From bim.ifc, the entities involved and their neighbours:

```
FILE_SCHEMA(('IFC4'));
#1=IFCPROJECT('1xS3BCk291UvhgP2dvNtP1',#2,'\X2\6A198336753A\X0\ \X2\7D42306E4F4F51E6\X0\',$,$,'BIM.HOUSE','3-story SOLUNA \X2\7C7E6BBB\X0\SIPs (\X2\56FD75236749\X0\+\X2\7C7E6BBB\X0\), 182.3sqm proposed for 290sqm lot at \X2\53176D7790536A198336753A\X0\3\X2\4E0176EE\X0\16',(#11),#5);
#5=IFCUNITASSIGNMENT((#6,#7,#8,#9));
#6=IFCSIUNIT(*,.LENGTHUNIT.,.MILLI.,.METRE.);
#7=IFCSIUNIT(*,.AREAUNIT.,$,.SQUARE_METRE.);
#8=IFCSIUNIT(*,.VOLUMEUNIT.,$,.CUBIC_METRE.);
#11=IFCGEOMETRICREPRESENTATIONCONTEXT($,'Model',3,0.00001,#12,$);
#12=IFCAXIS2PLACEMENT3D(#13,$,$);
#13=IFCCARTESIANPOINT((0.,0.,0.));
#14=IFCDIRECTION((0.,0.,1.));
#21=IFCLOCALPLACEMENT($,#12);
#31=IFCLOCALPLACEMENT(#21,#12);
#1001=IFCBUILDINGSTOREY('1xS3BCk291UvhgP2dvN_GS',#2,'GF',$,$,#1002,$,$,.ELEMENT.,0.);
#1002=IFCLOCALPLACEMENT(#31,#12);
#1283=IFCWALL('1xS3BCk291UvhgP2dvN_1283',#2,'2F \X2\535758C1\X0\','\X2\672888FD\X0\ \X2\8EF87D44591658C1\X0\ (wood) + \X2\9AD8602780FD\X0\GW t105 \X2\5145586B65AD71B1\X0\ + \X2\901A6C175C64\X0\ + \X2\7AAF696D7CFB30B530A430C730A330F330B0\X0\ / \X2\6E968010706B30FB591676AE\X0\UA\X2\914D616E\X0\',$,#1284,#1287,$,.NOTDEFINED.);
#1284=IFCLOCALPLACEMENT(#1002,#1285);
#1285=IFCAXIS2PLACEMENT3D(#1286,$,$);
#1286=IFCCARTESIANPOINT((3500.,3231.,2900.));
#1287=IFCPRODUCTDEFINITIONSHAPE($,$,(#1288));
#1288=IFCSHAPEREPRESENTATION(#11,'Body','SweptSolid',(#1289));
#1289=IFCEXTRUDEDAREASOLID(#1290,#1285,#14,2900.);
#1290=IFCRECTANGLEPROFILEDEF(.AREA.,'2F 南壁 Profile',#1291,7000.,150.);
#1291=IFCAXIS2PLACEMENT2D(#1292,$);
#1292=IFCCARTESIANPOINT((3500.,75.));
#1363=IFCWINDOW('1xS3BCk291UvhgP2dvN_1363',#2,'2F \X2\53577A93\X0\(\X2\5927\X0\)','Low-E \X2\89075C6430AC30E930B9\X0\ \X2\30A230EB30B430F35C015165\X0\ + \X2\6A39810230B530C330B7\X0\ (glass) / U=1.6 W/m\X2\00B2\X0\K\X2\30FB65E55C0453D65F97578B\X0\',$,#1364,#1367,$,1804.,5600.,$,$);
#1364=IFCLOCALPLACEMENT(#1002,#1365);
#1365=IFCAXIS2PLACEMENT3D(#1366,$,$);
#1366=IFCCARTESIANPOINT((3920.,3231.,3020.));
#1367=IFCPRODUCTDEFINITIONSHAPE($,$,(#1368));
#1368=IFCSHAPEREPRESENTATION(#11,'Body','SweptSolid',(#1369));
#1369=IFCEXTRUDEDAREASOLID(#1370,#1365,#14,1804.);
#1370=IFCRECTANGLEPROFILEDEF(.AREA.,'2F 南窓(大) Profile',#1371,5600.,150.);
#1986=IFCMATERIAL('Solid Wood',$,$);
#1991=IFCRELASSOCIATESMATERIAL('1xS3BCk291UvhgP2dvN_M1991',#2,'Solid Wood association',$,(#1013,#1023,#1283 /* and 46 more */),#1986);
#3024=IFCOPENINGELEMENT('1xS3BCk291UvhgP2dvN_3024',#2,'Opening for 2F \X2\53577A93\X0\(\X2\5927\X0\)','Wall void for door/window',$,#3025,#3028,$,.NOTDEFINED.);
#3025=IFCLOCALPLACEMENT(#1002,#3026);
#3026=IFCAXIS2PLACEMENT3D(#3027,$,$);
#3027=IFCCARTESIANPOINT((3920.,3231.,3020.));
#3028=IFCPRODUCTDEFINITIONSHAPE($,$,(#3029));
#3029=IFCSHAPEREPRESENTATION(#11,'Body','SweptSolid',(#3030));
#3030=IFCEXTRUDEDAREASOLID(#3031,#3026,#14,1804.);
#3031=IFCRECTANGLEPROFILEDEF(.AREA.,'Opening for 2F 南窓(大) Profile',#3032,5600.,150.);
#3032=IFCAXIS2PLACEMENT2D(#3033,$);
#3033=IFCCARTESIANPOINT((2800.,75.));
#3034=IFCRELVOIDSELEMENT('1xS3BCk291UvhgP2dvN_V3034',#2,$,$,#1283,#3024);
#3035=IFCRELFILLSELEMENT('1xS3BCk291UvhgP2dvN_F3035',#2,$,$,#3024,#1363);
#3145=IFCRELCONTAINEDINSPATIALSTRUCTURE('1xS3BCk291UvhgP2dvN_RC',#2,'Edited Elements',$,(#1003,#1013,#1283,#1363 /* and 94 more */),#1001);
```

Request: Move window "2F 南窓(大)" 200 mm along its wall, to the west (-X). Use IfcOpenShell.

```python
import ifcopenshell
import ifcopenshell.api.geometry
import ifcopenshell.util.placement

model = ifcopenshell.open("bim.ifc")

window = model.by_guid("1xS3BCk291UvhgP2dvN_1363")
opening = window.FillsVoids[0].RelatingOpeningElement
wall = opening.VoidsElements[0].RelatingBuildingElement

wall_matrix = ifcopenshell.util.placement.get_local_placement(wall.ObjectPlacement)
shift = wall_matrix[:3, 0] * -200.0
before = ifcopenshell.util.placement.get_local_placement(window.ObjectPlacement)[:3, 3].copy()

# The window is not placed relative to its opening, so move both.
for product in (opening, window):
    matrix = ifcopenshell.util.placement.get_local_placement(product.ObjectPlacement)
    matrix[:3, 3] += shift
    ifcopenshell.api.geometry.edit_object_placement(model, product=product, matrix=matrix, is_si=False)

after = ifcopenshell.util.placement.get_local_placement(window.ObjectPlacement)[:3, 3]
print("window moved by", (after - before).round(3) + 0.0)

model.write("bim_edited.ifc")
```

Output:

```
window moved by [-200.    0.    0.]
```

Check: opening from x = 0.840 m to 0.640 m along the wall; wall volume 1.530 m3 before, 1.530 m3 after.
